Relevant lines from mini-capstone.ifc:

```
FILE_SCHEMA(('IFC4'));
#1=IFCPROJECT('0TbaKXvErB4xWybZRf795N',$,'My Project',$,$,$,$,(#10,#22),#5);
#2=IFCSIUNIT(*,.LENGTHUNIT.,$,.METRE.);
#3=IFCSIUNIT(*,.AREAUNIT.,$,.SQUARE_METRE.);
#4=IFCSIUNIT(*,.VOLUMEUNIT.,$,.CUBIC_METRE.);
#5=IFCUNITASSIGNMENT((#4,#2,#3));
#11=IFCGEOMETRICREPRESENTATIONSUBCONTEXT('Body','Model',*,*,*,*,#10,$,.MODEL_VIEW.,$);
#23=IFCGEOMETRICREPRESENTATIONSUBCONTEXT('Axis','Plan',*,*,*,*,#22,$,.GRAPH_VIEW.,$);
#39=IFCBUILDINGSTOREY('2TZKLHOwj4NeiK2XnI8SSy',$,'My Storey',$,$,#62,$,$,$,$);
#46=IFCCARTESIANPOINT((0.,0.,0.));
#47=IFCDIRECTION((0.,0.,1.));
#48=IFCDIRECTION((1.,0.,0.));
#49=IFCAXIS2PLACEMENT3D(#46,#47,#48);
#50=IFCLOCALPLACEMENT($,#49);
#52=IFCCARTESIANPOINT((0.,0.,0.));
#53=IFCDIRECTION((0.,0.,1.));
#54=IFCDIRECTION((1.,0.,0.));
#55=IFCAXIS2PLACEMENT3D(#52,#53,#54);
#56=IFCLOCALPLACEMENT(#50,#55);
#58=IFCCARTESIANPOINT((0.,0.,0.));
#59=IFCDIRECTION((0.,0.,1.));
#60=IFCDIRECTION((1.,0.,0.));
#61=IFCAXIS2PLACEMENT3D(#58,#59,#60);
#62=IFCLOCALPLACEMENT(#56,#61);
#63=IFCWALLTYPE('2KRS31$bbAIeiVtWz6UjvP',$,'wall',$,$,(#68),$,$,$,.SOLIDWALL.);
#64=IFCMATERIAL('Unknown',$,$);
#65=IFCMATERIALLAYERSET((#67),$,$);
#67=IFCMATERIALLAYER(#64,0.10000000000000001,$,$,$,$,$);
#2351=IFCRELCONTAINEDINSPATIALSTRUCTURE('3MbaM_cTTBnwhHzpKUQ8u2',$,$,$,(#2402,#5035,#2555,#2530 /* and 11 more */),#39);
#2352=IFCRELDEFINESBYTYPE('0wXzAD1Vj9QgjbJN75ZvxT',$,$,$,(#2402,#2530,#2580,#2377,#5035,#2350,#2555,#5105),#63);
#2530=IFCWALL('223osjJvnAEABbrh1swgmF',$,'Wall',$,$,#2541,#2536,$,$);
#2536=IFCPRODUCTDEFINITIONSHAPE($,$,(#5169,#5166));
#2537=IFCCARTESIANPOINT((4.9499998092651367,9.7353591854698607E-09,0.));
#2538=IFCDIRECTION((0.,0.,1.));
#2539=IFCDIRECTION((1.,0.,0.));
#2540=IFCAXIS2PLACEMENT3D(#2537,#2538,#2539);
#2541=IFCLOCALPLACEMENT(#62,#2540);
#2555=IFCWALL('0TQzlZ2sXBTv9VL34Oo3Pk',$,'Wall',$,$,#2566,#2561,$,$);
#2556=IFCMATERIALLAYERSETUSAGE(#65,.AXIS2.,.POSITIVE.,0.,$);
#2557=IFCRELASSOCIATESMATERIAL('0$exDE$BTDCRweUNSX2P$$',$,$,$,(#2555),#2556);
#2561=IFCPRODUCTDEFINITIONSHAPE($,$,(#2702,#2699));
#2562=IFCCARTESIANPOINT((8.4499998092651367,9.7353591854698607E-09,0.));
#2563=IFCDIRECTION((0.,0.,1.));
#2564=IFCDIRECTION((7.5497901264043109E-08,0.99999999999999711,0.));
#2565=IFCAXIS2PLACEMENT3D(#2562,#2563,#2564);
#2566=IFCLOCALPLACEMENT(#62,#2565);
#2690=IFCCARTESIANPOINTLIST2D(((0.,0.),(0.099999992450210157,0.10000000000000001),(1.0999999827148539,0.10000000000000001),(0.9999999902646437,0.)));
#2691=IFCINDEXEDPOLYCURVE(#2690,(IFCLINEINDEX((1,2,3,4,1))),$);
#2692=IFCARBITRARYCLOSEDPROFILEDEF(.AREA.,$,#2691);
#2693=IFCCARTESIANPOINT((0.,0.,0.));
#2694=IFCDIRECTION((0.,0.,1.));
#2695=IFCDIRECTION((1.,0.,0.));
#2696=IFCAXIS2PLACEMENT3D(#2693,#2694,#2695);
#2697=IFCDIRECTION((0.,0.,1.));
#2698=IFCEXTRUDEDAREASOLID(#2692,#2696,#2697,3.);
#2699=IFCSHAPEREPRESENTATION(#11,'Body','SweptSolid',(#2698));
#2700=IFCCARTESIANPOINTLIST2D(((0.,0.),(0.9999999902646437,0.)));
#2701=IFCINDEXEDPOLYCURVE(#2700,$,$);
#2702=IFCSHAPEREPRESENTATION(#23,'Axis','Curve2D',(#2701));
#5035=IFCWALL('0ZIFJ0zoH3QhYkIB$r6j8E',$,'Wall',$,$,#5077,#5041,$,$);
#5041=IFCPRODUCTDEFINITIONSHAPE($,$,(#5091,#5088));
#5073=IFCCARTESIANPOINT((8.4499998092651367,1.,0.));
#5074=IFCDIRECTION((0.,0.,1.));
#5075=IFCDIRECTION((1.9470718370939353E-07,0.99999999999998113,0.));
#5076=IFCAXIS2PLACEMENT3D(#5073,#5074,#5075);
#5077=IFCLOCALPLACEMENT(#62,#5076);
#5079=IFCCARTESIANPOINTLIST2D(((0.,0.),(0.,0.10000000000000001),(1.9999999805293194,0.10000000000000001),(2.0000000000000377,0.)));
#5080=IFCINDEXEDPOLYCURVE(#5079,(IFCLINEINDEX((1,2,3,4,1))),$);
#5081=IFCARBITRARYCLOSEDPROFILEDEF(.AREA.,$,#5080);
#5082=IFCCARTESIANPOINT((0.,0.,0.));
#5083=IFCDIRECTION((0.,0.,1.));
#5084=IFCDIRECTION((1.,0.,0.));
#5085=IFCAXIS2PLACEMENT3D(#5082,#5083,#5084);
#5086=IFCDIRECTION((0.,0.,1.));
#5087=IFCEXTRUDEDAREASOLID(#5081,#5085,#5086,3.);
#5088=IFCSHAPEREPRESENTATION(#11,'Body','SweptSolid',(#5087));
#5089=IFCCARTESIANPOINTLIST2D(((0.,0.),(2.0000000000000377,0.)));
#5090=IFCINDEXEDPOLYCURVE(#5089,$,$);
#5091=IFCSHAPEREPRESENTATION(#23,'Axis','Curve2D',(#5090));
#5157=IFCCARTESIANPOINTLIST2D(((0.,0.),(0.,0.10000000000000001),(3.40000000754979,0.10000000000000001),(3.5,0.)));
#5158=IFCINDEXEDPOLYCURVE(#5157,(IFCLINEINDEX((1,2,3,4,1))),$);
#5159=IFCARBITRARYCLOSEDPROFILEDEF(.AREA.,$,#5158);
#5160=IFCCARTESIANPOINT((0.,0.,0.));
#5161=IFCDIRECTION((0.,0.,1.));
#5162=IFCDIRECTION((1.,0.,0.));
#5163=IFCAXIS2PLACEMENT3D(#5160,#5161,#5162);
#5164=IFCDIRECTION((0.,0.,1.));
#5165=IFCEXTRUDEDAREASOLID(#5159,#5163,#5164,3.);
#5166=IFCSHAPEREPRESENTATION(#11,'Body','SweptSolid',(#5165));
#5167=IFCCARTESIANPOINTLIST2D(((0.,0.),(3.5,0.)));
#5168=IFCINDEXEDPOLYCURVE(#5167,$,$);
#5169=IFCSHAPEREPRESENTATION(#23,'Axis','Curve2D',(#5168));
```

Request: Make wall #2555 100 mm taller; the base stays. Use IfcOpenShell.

```python
import ifcopenshell
import ifcopenshell.geom
import ifcopenshell.util.representation
import ifcopenshell.util.shape
import ifcopenshell.util.unit

model = ifcopenshell.open("mini-capstone.ifc")
unit_scale = ifcopenshell.util.unit.calculate_unit_scale(model)
settings = ifcopenshell.geom.settings()


def volume(element):
    """Net volume in cubic metres, openings subtracted."""
    shape = ifcopenshell.geom.create_shape(settings, element)
    return ifcopenshell.util.shape.get_volume(shape.geometry)


wall = model.by_id(2555)
before = volume(wall)

body = ifcopenshell.util.representation.get_representation(wall, "Model", "Body")
solid = body.Items[0]
old_height = solid.Depth
solid.Depth += 0.1 / unit_scale
after = volume(wall)

print(f"height {old_height:g} -> {solid.Depth:g}, volume {before:.3f} -> {after:.3f} m3")

model.write("mini-capstone_rev.ifc")
```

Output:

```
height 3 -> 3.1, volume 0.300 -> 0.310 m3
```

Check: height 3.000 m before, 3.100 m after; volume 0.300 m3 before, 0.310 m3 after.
